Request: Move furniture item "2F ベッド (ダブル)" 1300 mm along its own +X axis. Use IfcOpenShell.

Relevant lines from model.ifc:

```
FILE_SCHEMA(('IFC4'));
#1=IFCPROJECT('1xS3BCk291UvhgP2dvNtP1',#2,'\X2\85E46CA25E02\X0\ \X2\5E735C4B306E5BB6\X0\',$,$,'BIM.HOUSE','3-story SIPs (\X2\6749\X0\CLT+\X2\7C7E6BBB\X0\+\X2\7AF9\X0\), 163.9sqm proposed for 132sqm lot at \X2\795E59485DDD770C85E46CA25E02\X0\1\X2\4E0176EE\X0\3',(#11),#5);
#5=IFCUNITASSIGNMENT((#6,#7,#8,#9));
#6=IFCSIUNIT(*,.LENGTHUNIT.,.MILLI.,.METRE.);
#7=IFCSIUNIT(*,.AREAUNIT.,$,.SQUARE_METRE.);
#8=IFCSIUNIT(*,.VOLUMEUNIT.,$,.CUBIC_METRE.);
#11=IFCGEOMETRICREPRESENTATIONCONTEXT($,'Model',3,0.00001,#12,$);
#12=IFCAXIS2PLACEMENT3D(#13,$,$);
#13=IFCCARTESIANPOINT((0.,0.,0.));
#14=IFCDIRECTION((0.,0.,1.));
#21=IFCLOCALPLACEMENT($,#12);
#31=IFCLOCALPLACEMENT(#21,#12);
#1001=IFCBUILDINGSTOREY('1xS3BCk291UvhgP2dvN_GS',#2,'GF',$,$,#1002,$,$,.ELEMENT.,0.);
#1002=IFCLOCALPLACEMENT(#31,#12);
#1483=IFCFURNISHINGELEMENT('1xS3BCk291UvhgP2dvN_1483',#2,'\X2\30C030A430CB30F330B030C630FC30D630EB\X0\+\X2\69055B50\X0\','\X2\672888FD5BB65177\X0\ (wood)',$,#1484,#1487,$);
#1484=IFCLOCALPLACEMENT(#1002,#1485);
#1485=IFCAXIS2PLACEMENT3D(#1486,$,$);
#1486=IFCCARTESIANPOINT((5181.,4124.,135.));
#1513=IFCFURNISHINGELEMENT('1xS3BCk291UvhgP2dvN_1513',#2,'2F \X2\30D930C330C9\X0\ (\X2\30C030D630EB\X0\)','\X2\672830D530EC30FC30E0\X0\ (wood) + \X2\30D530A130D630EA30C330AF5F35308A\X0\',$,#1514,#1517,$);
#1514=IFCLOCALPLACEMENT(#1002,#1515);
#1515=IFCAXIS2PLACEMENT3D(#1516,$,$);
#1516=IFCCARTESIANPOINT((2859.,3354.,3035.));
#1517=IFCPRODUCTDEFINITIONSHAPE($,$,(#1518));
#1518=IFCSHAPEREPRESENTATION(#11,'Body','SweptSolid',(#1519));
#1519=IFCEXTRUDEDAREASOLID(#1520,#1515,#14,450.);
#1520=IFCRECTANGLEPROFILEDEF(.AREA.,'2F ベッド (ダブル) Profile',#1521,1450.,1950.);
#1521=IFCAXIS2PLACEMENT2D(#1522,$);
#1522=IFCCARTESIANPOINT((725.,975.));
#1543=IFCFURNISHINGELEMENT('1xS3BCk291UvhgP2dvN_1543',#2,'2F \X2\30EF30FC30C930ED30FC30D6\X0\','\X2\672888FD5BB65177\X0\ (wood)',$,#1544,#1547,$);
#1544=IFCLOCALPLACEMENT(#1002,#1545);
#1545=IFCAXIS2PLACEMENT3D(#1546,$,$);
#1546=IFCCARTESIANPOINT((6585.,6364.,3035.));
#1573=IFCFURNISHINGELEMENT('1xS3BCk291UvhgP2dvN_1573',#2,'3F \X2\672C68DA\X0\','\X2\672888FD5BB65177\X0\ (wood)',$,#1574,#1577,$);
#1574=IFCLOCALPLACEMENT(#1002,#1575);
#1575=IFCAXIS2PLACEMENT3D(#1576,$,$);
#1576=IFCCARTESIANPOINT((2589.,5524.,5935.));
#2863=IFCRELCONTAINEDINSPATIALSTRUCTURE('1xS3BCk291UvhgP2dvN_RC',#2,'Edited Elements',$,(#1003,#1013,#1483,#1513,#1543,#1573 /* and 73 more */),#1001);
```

```python
import ifcopenshell
import ifcopenshell.api.geometry
import ifcopenshell.util.placement
import ifcopenshell.util.unit

model = ifcopenshell.open("model.ifc")
unit_scale = ifcopenshell.util.unit.calculate_unit_scale(model)

item = model.by_guid("1xS3BCk291UvhgP2dvN_1513")
matrix = ifcopenshell.util.placement.get_local_placement(item.ObjectPlacement)
matrix[:3, 3] += matrix[:3, 0] * 1.3 / unit_scale
ifcopenshell.api.geometry.edit_object_placement(model, product=item, matrix=matrix, is_si=False)

print(ifcopenshell.util.placement.get_local_placement(item.ObjectPlacement).round(3) + 0.0)

model.write("model_edited.ifc")
```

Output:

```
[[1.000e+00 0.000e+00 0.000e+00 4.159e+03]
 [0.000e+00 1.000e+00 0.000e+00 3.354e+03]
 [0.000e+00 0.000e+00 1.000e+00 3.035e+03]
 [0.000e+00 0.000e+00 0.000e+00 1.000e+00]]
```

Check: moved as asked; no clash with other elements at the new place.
